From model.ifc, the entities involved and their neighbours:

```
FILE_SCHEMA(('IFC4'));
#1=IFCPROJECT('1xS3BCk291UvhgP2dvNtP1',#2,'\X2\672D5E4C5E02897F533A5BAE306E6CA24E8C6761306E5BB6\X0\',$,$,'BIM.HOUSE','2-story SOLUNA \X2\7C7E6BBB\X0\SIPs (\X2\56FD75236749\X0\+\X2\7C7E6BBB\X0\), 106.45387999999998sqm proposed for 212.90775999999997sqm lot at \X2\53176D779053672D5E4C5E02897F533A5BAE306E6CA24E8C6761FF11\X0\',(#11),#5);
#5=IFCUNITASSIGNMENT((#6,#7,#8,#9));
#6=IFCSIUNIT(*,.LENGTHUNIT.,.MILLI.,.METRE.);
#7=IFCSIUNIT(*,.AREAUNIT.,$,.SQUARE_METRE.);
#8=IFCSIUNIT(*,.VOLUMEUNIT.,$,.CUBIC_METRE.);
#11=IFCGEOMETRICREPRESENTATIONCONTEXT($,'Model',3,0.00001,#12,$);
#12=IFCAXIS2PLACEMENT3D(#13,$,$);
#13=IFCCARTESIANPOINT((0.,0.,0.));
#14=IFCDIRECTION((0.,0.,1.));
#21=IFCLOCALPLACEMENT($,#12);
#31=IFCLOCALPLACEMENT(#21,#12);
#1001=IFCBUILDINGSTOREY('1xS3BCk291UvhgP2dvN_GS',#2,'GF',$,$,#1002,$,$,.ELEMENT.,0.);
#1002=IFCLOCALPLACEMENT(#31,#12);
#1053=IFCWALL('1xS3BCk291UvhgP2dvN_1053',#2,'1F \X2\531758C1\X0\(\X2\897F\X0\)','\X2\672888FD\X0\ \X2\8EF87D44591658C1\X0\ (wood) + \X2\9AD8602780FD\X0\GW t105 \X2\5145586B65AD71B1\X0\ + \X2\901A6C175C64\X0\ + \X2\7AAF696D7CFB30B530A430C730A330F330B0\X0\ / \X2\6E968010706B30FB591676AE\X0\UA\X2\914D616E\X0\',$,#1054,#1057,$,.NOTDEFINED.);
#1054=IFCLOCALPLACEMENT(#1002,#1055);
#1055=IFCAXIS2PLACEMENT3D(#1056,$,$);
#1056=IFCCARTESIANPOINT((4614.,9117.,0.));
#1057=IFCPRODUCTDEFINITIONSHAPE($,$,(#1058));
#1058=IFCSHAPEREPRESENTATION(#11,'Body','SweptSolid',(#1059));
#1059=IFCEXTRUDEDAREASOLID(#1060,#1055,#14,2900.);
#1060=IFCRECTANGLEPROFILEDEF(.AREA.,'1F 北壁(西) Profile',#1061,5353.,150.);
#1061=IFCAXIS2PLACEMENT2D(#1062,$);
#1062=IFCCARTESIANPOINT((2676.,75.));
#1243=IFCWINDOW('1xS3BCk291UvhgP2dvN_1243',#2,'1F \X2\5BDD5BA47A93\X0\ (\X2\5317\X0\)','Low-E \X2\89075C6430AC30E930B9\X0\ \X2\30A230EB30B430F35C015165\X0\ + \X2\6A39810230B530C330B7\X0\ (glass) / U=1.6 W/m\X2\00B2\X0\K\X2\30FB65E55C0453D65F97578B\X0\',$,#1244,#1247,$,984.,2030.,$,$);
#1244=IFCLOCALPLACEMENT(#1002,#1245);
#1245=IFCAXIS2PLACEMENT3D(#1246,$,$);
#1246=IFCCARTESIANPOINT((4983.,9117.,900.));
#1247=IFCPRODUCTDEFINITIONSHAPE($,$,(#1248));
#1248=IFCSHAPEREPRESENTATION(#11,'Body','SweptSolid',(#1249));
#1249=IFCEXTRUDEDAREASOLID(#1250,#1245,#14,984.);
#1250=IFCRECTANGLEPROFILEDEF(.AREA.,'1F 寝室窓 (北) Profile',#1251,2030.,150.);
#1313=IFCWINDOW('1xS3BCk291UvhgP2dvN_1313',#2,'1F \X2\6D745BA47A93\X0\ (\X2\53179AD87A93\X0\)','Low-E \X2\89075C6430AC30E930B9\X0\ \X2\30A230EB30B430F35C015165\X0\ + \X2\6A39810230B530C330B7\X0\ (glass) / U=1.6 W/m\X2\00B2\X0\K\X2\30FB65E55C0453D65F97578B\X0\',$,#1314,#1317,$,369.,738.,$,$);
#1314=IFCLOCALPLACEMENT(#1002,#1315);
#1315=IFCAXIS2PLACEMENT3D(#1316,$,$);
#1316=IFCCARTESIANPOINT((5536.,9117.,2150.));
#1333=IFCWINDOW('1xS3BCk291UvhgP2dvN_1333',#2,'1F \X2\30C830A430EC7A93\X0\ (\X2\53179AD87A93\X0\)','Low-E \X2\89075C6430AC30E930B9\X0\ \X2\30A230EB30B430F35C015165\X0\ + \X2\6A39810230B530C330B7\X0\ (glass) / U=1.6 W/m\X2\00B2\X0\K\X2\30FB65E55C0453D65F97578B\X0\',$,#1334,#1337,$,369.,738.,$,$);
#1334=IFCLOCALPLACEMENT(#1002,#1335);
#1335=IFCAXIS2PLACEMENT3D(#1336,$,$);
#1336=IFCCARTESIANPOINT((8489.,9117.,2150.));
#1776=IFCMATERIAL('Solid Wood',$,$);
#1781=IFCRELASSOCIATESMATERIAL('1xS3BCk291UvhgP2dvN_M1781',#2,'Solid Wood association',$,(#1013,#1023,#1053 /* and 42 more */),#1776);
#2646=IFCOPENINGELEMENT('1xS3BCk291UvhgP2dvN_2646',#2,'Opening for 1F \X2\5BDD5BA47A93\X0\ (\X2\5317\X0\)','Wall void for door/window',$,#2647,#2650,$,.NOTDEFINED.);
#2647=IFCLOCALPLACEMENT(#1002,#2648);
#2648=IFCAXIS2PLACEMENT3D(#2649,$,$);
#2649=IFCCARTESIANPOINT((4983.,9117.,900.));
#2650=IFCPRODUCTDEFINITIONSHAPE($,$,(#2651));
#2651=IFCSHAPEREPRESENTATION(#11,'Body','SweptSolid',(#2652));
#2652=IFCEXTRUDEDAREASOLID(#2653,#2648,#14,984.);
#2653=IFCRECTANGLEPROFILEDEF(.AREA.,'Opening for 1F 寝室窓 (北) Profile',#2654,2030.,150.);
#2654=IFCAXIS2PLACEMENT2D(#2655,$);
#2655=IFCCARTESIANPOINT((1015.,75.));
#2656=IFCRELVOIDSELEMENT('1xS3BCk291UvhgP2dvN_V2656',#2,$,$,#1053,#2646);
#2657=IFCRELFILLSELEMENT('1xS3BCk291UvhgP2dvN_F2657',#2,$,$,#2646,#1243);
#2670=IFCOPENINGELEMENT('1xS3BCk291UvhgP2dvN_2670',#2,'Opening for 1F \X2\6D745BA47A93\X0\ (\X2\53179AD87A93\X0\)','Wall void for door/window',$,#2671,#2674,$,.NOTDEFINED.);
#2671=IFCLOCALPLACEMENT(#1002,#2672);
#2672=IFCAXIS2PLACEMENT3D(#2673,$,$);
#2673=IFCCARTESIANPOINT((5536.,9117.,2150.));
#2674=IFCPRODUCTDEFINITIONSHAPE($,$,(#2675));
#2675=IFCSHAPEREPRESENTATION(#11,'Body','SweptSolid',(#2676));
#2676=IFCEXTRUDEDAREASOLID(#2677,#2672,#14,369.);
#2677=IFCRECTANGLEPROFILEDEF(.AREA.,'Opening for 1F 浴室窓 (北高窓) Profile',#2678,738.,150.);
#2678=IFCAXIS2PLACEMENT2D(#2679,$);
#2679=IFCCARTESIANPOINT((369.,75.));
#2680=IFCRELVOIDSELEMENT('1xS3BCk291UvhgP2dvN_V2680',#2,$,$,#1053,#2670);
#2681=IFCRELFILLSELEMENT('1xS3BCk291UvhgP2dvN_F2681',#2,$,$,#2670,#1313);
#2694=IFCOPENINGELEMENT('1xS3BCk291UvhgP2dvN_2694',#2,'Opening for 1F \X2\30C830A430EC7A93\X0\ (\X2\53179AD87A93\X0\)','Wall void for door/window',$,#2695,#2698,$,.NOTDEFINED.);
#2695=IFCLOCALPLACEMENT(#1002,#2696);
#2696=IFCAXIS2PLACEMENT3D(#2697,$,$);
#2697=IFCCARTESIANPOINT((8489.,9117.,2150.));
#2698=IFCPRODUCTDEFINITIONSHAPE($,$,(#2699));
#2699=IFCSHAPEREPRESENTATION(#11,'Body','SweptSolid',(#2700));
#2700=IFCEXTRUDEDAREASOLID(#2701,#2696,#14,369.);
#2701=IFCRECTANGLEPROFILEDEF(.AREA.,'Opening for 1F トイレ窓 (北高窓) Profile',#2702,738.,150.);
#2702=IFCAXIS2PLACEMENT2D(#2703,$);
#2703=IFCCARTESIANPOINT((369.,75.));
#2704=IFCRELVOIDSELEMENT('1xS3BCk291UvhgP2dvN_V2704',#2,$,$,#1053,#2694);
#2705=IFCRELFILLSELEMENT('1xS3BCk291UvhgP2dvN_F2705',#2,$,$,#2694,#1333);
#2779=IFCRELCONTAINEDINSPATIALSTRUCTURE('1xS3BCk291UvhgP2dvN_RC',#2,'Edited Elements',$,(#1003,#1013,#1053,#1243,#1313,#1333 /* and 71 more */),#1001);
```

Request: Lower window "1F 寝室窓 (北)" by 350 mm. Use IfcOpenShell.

```python
import numpy as np
import ifcopenshell
import ifcopenshell.api.geometry
import ifcopenshell.util.placement
import ifcopenshell.util.unit

model = ifcopenshell.open("model.ifc")
unit_scale = ifcopenshell.util.unit.calculate_unit_scale(model)

window = model.by_id(1243)
opening = window.FillsVoids[0].RelatingOpeningElement
dz = -0.35 / unit_scale

shift = np.array([0.0, 0.0, dz])
# The window is not placed relative to its opening, so move both.
for product in (opening, window):
    matrix = ifcopenshell.util.placement.get_local_placement(product.ObjectPlacement)
    matrix[:3, 3] += shift
    ifcopenshell.api.geometry.edit_object_placement(model, product=product, matrix=matrix, is_si=False)

print(f"moved by {dz * unit_scale:+.3f} m")

model.write("model_updated.ifc")
```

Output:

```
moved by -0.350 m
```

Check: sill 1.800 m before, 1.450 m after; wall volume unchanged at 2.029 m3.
